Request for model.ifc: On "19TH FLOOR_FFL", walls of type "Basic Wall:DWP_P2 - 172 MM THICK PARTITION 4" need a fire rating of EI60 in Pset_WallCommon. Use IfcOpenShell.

First a look at what the model holds.

```python
import ifcopenshell
import ifcopenshell.util.element

model = ifcopenshell.open("model.ifc")
print(model.schema)
storey = next(s for s in model.by_type("IfcBuildingStorey") if s.Name == "19TH FLOOR_FFL")
walls = [e for e in ifcopenshell.util.element.get_decomposition(storey) if e.is_a("IfcWall")]
seen = {}
for e in walls:
    element_type = ifcopenshell.util.element.get_type(e)
    key = (element_type.Name if element_type != e and element_type else None, ifcopenshell.util.element.get_pset(e, "Pset_WallCommon", "FireRating"))
    seen[key] = seen.get(key, 0) + 1
for (name, value), count in sorted(seen.items(), key=str):
    print(count, "x", name, "|", value)
```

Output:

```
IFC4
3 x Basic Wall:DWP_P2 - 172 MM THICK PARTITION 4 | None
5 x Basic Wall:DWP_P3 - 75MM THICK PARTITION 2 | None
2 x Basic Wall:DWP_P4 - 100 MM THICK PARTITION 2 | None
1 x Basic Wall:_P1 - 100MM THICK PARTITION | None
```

```python
import ifcopenshell
import ifcopenshell.api.pset
import ifcopenshell.util.element

model = ifcopenshell.open("model.ifc")

storey = next(s for s in model.by_type("IfcBuildingStorey") if s.Name == "19TH FLOOR_FFL")
walls = [e for e in ifcopenshell.util.element.get_decomposition(storey) if e.is_a("IfcWall")]

count = 0
for e in walls:
    element_type = ifcopenshell.util.element.get_type(e)
    if element_type in (None, e) or element_type.Name != "Basic Wall:DWP_P2 - 172 MM THICK PARTITION 4":
        continue
    # add_pset returns the element's existing set when there is one.
    pset = ifcopenshell.api.pset.add_pset(model, product=e, name="Pset_WallCommon")
    ifcopenshell.api.pset.edit_pset(model, pset=pset, properties={"FireRating": "EI60"})
    count += 1

print(count, "walls updated")

model.write("model_v2.ifc")
```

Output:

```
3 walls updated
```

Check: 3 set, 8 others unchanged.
